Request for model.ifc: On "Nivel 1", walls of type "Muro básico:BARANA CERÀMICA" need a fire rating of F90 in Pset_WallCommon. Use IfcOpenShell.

First a look at what the model holds.

```python
import ifcopenshell
import ifcopenshell.util.element

model = ifcopenshell.open("model.ifc")
print(model.schema)
storey = next(s for s in model.by_type("IfcBuildingStorey") if s.Name == "Nivel 1")
walls = [e for e in ifcopenshell.util.element.get_decomposition(storey) if e.is_a("IfcWall")]
seen = {}
for e in walls:
    element_type = ifcopenshell.util.element.get_type(e)
    key = (element_type.Name if element_type != e and element_type else None, ifcopenshell.util.element.get_pset(e, "Pset_WallCommon", "FireRating"))
    seen[key] = seen.get(key, 0) + 1
for (name, value), count in sorted(seen.items(), key=str):
    print(count, "x", name, "|", value)
```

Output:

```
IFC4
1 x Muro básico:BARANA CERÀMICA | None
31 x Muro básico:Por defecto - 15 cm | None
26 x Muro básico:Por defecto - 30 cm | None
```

```python
import ifcopenshell
import ifcopenshell.api.pset
import ifcopenshell.util.element

model = ifcopenshell.open("model.ifc")

storey = next(s for s in model.by_type("IfcBuildingStorey") if s.Name == "Nivel 1")
walls = [e for e in ifcopenshell.util.element.get_decomposition(storey) if e.is_a("IfcWall")]

count = 0
for e in walls:
    element_type = ifcopenshell.util.element.get_type(e)
    if element_type in (None, e) or element_type.Name != "Muro básico:BARANA CERÀMICA":
        continue
    # add_pset returns the element's existing set when there is one.
    pset = ifcopenshell.api.pset.add_pset(model, product=e, name="Pset_WallCommon")
    ifcopenshell.api.pset.edit_pset(model, pset=pset, properties={"FireRating": "F90"})
    count += 1

print(count, "walls updated")

model.write("model_rev.ifc")
```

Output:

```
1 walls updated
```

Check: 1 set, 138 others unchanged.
